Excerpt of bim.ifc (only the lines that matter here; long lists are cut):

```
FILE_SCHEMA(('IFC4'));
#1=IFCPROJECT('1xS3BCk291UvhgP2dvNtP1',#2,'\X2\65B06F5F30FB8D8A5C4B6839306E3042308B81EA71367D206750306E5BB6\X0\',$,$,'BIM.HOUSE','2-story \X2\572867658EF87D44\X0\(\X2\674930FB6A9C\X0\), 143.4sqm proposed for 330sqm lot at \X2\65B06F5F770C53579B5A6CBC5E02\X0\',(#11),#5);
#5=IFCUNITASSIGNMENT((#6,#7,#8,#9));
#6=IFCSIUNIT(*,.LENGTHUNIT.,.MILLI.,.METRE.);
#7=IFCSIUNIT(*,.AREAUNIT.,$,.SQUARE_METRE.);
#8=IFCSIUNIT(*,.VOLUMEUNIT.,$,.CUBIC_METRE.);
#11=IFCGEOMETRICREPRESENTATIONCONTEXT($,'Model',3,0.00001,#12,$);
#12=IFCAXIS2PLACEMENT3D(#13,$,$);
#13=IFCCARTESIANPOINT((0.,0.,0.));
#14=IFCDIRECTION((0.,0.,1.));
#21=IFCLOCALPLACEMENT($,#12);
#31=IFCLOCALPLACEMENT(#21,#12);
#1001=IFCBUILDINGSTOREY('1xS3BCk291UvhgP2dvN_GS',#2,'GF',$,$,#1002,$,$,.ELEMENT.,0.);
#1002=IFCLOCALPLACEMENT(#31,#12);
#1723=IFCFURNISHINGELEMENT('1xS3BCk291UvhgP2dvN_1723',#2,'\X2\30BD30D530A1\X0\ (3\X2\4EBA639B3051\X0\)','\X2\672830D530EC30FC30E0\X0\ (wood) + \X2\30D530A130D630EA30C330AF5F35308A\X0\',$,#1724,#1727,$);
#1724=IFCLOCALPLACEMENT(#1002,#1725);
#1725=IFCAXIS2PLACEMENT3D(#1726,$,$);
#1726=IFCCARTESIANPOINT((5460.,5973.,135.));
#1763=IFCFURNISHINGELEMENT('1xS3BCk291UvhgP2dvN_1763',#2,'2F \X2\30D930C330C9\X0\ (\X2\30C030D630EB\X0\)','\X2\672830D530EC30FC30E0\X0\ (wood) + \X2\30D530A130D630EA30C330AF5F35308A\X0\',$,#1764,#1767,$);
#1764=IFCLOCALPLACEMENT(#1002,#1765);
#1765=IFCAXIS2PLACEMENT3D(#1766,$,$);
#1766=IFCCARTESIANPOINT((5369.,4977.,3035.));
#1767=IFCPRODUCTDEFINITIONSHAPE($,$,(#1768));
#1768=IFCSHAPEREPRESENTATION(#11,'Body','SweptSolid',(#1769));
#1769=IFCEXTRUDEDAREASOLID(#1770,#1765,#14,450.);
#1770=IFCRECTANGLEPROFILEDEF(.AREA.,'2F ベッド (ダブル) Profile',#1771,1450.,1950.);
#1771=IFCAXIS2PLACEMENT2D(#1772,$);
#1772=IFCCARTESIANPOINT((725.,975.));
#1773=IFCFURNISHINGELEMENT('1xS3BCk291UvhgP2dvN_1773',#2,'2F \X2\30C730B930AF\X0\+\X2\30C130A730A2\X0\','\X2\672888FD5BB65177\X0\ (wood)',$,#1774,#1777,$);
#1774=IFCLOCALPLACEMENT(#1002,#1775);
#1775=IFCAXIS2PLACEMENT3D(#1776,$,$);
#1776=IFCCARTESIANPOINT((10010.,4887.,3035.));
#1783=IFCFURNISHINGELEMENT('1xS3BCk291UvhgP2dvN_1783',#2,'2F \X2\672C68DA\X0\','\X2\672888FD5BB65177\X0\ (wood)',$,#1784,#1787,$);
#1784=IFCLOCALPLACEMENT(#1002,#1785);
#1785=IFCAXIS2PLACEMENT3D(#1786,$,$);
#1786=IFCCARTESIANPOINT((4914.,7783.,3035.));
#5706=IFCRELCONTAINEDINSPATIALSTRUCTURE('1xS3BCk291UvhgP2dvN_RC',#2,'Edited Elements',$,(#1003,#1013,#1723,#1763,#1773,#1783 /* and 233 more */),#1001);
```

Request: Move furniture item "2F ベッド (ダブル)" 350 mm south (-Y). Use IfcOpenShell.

```python
import ifcopenshell
import ifcopenshell.api.geometry
import ifcopenshell.util.placement
import ifcopenshell.util.unit

model = ifcopenshell.open("bim.ifc")
unit_scale = ifcopenshell.util.unit.calculate_unit_scale(model)

item = model.by_guid("1xS3BCk291UvhgP2dvN_1763")
matrix = ifcopenshell.util.placement.get_local_placement(item.ObjectPlacement)
matrix[1, 3] -= 0.35 / unit_scale
ifcopenshell.api.geometry.edit_object_placement(model, product=item, matrix=matrix, is_si=False)

print(ifcopenshell.util.placement.get_local_placement(item.ObjectPlacement).round(3) + 0.0)

model.write("bim_updated.ifc")
```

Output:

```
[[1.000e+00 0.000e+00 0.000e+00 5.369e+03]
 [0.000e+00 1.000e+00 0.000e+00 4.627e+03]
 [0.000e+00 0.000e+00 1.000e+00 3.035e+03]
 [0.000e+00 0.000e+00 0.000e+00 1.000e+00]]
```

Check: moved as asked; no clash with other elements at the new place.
